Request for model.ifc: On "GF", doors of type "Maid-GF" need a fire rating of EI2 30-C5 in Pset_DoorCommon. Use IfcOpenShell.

First a look at what the model holds.

```python
import ifcopenshell
import ifcopenshell.util.element

model = ifcopenshell.open("model.ifc")
print(model.schema)
storey = next(s for s in model.by_type("IfcBuildingStorey") if s.Name == "GF")
doors = [e for e in ifcopenshell.util.element.get_decomposition(storey) if e.is_a("IfcDoor")]
seen = {}
for e in doors:
    element_type = ifcopenshell.util.element.get_type(e)
    key = (element_type.Name if element_type != e and element_type else None, ifcopenshell.util.element.get_pset(e, "Pset_DoorCommon", "FireRating"))
    seen[key] = seen.get(key, 0) + 1
for (name, value), count in sorted(seen.items(), key=str):
    print(count, "x", name, "|", value)
```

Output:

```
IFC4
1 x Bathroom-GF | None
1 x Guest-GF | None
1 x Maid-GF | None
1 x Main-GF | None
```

```python
import ifcopenshell
import ifcopenshell.api.pset
import ifcopenshell.util.element

model = ifcopenshell.open("model.ifc")

storey = next(s for s in model.by_type("IfcBuildingStorey") if s.Name == "GF")
doors = [e for e in ifcopenshell.util.element.get_decomposition(storey) if e.is_a("IfcDoor")]

count = 0
for e in doors:
    element_type = ifcopenshell.util.element.get_type(e)
    if element_type in (None, e) or element_type.Name != "Maid-GF":
        continue
    # add_pset returns the element's existing set when there is one.
    pset = ifcopenshell.api.pset.add_pset(model, product=e, name="Pset_DoorCommon")
    ifcopenshell.api.pset.edit_pset(model, pset=pset, properties={"FireRating": "EI2 30-C5"})
    count += 1

print(count, "doors updated")

model.write("model_updated.ifc")
```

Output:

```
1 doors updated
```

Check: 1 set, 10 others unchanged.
